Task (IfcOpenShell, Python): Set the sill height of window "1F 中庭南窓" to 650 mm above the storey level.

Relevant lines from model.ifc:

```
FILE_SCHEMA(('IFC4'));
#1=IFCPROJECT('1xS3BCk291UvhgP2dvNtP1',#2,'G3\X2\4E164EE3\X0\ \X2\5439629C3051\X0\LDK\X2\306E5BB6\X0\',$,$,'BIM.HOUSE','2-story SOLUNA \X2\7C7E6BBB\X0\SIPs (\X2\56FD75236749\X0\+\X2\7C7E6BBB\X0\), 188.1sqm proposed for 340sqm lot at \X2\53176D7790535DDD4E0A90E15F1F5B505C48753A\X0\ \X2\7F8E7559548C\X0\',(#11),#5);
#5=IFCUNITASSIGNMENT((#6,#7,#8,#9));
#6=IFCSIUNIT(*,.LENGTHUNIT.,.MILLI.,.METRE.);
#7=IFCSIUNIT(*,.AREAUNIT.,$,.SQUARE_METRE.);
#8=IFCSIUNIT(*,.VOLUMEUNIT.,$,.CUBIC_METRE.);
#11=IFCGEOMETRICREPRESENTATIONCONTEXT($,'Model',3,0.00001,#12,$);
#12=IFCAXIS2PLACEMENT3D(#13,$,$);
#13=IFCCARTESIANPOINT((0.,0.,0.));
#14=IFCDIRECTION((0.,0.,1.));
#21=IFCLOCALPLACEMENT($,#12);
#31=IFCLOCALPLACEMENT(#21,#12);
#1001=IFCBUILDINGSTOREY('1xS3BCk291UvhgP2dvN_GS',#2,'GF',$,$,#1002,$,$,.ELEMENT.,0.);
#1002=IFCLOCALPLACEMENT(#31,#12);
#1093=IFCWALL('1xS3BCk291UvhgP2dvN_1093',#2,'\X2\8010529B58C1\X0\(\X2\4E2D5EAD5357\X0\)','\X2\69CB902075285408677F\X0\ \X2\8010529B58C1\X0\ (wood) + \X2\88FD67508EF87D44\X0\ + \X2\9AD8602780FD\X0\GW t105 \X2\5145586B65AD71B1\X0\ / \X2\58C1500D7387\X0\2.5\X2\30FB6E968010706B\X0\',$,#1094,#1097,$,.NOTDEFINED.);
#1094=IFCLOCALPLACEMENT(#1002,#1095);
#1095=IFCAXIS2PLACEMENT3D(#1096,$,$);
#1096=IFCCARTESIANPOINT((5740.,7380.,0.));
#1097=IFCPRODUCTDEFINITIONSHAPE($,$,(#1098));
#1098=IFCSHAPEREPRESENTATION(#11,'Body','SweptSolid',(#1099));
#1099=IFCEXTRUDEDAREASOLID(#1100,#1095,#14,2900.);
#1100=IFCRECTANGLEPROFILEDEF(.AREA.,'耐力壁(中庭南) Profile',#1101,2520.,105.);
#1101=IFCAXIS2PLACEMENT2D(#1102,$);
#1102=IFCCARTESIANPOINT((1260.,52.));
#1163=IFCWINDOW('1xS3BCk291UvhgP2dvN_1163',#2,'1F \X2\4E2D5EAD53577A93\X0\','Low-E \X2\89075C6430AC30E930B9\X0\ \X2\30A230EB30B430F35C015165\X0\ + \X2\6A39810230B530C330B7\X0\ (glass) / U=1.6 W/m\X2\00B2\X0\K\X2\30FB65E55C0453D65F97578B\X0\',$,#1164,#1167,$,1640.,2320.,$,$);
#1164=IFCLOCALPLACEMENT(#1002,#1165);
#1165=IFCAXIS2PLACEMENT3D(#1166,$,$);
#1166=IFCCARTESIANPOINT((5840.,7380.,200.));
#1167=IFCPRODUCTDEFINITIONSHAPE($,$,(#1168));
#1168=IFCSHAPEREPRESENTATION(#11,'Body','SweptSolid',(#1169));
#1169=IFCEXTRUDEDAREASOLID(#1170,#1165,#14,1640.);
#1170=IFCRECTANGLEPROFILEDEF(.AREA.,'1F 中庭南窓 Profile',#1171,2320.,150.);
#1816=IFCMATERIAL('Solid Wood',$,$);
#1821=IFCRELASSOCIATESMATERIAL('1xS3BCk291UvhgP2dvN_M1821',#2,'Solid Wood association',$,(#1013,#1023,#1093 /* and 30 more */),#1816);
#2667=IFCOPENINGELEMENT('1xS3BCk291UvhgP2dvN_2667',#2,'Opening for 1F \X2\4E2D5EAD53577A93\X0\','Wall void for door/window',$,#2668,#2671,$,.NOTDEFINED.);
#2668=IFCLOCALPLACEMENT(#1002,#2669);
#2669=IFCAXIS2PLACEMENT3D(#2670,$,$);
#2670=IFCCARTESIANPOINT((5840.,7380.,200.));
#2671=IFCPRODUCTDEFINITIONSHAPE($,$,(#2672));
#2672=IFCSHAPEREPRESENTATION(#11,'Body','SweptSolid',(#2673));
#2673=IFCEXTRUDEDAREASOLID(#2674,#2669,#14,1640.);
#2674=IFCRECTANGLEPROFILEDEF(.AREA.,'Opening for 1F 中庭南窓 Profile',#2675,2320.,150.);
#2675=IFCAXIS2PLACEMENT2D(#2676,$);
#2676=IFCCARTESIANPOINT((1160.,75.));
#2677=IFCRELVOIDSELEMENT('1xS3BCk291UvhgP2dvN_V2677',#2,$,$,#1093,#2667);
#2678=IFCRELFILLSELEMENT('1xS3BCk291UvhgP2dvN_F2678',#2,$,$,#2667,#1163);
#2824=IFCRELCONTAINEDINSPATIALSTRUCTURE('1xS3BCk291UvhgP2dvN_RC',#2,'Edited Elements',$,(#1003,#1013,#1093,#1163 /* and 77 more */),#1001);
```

```python
import numpy as np
import ifcopenshell
import ifcopenshell.api.geometry
import ifcopenshell.geom
import ifcopenshell.util.element
import ifcopenshell.util.placement
import ifcopenshell.util.shape
import ifcopenshell.util.unit

model = ifcopenshell.open("model.ifc")
unit_scale = ifcopenshell.util.unit.calculate_unit_scale(model)

window = model.by_guid("1xS3BCk291UvhgP2dvN_1163")
opening = window.FillsVoids[0].RelatingOpeningElement
storey = ifcopenshell.util.element.get_container(window, ifc_class="IfcBuildingStorey")
level = ifcopenshell.util.placement.get_local_placement(storey.ObjectPlacement)[2, 3]

# The opening's origin need not be at the sill, so measure its lowest point.
shape = ifcopenshell.geom.create_shape(ifcopenshell.geom.settings(), opening)
bottom = ifcopenshell.util.shape.get_shape_bottom_elevation(shape, shape.geometry) / unit_scale
dz = level + 650.0 - bottom

shift = np.array([0.0, 0.0, dz])
# The window is not placed relative to its opening, so move both.
for product in (opening, window):
    matrix = ifcopenshell.util.placement.get_local_placement(product.ObjectPlacement)
    matrix[:3, 3] += shift
    ifcopenshell.api.geometry.edit_object_placement(model, product=product, matrix=matrix, is_si=False)

print(f"moved by {dz * unit_scale:+.3f} m")

model.write("model-out.ifc")
```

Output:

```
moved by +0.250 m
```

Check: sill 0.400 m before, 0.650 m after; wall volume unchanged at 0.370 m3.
